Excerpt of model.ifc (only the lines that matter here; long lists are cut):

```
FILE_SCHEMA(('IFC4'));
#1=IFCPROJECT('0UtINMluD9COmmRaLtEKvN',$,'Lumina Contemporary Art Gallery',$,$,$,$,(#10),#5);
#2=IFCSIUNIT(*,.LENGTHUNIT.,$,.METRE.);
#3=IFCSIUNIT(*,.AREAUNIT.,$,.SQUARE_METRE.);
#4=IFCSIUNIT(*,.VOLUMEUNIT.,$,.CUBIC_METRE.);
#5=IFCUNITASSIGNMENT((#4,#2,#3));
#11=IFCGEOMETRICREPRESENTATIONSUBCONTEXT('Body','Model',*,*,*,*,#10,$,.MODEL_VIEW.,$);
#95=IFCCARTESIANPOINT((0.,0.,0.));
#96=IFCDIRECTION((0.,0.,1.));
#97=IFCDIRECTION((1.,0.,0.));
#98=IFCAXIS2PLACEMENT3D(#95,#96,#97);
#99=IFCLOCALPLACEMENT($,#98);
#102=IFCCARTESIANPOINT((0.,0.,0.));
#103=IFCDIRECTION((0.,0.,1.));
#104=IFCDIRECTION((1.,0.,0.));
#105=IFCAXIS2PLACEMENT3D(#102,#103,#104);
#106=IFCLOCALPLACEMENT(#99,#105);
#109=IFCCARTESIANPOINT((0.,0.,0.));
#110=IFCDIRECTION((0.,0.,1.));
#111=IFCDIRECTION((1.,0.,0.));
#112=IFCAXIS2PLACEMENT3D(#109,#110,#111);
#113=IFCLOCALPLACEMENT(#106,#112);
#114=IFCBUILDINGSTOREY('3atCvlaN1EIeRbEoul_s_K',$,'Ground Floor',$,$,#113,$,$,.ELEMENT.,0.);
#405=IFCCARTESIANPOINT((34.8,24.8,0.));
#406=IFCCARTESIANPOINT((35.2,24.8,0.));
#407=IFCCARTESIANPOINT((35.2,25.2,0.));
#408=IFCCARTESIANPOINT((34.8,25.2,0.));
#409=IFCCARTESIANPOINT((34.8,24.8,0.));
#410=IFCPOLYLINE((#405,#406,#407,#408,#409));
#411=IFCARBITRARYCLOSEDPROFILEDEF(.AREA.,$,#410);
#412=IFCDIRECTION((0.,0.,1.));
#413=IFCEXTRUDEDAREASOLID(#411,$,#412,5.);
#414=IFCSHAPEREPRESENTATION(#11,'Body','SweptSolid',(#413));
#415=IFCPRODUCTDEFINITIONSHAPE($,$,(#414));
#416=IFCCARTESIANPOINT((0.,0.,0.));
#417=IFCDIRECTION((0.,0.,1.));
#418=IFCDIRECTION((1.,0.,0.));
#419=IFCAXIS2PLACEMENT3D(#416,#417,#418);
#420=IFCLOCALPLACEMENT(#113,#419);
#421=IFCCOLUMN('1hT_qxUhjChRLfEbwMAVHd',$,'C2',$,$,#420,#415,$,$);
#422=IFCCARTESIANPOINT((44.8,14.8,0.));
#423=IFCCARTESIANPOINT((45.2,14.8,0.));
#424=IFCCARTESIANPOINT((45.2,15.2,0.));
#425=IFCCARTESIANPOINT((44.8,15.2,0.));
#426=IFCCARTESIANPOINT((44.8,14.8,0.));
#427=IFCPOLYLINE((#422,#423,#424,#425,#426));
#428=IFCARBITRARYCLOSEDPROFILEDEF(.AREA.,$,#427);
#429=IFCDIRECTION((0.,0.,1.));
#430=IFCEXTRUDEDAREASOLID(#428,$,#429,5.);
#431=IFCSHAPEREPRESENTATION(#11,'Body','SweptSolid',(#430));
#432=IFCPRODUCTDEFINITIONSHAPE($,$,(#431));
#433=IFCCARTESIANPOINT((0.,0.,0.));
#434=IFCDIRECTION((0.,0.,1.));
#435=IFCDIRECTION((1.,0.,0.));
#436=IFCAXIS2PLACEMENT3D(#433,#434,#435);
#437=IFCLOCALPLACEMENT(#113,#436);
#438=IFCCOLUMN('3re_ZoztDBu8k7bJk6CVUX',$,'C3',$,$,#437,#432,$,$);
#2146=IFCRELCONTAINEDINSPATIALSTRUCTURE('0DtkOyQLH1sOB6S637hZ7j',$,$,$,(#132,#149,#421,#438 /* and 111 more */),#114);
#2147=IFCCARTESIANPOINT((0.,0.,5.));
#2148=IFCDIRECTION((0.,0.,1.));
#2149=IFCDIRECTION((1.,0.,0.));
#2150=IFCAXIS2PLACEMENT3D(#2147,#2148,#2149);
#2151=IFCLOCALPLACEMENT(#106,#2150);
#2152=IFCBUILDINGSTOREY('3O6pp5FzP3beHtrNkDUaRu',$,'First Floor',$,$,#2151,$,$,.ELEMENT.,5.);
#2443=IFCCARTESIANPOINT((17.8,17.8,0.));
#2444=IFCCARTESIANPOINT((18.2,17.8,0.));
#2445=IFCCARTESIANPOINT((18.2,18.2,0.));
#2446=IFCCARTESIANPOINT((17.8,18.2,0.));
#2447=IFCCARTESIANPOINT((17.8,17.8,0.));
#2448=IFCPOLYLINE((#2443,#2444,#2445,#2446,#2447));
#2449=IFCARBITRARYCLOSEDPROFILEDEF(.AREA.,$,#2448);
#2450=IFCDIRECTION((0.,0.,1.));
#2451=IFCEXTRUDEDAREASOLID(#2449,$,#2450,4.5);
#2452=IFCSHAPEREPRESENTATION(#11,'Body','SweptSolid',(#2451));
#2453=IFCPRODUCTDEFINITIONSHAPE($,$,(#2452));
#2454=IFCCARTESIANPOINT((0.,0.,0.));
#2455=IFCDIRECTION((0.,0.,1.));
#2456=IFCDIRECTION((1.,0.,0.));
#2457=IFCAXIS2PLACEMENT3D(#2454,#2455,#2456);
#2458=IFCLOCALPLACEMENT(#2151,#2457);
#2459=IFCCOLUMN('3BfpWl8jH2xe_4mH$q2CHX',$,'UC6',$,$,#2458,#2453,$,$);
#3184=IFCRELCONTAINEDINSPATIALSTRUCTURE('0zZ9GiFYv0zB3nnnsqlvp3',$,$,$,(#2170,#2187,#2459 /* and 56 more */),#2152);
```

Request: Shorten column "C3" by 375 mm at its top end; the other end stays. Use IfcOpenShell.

```python
import ifcopenshell
import ifcopenshell.util.representation
import ifcopenshell.util.unit

model = ifcopenshell.open("model.ifc")
unit_scale = ifcopenshell.util.unit.calculate_unit_scale(model)

member = model.by_id(438)
change = -0.375 / unit_scale

# The extrusion runs towards the end named, so only its depth changes.
body = ifcopenshell.util.representation.get_representation(member, "Model", "Body")
solid = body.Items[0]
old_length = solid.Depth
solid.Depth += change

print(f"length {old_length:g} -> {solid.Depth:g}")

model.write("model_edited.ifc")
```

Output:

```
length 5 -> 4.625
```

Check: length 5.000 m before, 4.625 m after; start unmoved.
